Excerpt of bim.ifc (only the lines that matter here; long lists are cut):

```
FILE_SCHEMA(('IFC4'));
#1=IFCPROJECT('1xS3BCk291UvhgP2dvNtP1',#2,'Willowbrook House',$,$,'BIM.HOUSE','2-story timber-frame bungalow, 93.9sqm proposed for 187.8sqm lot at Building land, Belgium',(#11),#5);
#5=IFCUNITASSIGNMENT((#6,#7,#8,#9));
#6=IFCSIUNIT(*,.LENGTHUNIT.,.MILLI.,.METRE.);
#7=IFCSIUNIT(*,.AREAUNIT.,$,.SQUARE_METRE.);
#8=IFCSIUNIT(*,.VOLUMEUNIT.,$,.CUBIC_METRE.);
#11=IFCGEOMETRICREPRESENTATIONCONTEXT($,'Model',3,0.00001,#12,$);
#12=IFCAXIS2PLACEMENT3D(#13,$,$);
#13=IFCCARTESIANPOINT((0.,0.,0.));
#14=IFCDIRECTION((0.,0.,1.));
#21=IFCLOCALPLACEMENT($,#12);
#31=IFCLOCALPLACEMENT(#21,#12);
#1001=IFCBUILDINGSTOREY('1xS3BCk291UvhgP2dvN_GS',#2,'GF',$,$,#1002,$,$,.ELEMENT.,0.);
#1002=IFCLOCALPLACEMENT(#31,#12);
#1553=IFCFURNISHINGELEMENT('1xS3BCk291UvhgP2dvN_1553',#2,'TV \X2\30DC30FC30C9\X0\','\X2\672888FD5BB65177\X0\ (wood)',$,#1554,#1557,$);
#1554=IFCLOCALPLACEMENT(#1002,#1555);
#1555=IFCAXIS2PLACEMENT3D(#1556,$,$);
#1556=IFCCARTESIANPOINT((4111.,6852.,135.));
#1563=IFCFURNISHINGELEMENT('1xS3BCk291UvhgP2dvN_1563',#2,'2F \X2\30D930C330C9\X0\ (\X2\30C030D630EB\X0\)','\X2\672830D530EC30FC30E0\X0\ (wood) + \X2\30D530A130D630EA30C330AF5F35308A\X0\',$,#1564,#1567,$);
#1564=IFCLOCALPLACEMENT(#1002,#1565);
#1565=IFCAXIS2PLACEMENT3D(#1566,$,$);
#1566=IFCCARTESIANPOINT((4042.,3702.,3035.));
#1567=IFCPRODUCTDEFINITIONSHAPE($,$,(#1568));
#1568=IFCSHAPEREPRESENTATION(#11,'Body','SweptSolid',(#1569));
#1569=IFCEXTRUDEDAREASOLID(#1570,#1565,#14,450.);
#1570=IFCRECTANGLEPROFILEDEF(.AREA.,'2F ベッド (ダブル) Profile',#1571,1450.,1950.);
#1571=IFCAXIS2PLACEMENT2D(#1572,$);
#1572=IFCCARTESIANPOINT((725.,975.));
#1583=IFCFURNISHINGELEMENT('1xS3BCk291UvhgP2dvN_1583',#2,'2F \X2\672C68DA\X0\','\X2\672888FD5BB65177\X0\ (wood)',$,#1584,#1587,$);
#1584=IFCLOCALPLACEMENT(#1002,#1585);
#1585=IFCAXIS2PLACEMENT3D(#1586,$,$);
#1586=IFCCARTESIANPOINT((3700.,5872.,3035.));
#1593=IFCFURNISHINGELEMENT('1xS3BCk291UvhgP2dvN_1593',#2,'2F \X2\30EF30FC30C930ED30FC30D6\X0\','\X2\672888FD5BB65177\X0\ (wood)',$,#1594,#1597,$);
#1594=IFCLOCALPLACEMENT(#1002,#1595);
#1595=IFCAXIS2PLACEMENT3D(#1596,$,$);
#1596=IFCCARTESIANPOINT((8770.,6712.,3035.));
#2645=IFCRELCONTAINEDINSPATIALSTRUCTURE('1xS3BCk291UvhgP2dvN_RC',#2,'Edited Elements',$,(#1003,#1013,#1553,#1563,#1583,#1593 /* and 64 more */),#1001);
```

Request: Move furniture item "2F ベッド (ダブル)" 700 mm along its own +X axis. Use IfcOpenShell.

```python
import ifcopenshell
import ifcopenshell.api.geometry
import ifcopenshell.util.placement
import ifcopenshell.util.unit

model = ifcopenshell.open("bim.ifc")
unit_scale = ifcopenshell.util.unit.calculate_unit_scale(model)

item = model.by_guid("1xS3BCk291UvhgP2dvN_1563")
matrix = ifcopenshell.util.placement.get_local_placement(item.ObjectPlacement)
matrix[:3, 3] += matrix[:3, 0] * 0.7 / unit_scale
ifcopenshell.api.geometry.edit_object_placement(model, product=item, matrix=matrix, is_si=False)

print(ifcopenshell.util.placement.get_local_placement(item.ObjectPlacement).round(3) + 0.0)

model.write("bim-out.ifc")
```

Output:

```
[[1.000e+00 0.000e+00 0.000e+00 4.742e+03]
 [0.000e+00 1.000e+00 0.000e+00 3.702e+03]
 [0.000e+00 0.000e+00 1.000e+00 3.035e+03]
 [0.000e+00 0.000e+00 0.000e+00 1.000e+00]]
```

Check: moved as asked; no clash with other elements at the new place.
